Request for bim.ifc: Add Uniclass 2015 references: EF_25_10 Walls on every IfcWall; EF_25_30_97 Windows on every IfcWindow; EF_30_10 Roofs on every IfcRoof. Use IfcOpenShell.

First a look at what the model holds.

```python
import ifcopenshell

model = ifcopenshell.open("bim.ifc")
print(model.schema)
print("classifications:", [c.Name for c in model.by_type("IfcClassification")])
for ifc_class in ("IfcDoor", "IfcRoof", "IfcStair", "IfcWall", "IfcWindow"):
    print(ifc_class, len(model.by_type(ifc_class)))
```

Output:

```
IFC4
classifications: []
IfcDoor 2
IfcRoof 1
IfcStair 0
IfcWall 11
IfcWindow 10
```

```python
import ifcopenshell
import ifcopenshell.api.classification

model = ifcopenshell.open("bim.ifc")

system = ifcopenshell.api.classification.add_classification(model, classification="Uniclass 2015")

codes = {
    "IfcWall": ("EF_25_10", "Walls"),
    "IfcWindow": ("EF_25_30_97", "Windows"),
    "IfcRoof": ("EF_30_10", "Roofs"),
}
for ifc_class, (code, name) in codes.items():
    products = model.by_type(ifc_class)
    ifcopenshell.api.classification.add_reference(
        model, products=products, classification=system, identification=code, name=name
    )
    print(code, len(products))

model.write("bim_updated.ifc")
```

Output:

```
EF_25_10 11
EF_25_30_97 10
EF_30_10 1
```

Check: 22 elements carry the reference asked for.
